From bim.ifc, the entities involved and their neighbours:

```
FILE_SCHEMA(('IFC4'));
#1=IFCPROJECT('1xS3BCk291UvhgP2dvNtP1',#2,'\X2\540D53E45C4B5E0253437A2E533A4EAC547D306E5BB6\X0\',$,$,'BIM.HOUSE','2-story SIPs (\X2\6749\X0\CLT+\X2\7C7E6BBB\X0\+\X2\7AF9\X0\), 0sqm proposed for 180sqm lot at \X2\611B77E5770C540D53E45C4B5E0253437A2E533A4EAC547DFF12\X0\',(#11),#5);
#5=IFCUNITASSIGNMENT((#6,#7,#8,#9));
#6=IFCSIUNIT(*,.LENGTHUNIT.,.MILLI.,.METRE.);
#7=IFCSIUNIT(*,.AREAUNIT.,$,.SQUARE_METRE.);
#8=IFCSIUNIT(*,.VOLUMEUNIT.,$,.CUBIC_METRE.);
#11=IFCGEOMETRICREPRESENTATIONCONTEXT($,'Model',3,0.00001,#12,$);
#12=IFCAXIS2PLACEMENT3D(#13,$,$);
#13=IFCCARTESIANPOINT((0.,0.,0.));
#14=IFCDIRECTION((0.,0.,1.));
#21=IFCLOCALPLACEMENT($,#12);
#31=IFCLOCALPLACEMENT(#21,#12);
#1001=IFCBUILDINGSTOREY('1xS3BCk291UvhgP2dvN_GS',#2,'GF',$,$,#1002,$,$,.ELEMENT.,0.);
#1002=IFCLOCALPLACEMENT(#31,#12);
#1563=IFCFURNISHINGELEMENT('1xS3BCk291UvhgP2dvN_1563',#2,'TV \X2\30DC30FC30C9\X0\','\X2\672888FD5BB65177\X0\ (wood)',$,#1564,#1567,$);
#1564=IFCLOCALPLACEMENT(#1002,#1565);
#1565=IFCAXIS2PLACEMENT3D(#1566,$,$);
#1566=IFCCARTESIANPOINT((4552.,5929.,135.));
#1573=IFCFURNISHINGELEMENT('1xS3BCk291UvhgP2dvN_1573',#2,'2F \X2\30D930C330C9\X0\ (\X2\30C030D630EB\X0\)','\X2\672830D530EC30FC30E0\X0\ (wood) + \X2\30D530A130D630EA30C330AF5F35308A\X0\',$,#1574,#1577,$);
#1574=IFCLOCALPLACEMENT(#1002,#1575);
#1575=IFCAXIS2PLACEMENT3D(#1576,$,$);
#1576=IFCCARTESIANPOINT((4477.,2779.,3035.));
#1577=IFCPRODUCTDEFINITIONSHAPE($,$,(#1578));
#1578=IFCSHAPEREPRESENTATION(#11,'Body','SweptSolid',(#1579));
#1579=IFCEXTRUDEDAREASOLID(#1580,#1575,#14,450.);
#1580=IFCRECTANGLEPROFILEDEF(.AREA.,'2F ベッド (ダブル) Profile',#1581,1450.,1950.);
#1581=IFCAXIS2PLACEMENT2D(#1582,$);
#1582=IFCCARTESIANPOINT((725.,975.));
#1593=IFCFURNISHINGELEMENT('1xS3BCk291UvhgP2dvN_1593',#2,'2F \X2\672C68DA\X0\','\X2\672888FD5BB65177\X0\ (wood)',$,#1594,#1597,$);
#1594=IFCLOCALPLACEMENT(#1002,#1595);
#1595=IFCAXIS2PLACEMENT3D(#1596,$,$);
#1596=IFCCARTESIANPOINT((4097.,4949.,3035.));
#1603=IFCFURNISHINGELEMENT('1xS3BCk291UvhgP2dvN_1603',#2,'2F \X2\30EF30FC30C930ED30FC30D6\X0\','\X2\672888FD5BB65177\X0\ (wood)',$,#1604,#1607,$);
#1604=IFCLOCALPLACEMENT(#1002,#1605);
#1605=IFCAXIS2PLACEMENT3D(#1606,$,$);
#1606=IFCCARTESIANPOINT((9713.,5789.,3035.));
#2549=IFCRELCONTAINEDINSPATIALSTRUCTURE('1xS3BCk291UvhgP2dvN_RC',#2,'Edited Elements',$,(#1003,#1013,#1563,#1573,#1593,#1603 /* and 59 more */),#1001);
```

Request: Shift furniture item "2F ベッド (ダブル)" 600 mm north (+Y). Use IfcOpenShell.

```python
import ifcopenshell
import ifcopenshell.api.geometry
import ifcopenshell.util.placement
import ifcopenshell.util.unit

model = ifcopenshell.open("bim.ifc")
unit_scale = ifcopenshell.util.unit.calculate_unit_scale(model)

item = model.by_guid("1xS3BCk291UvhgP2dvN_1573")
matrix = ifcopenshell.util.placement.get_local_placement(item.ObjectPlacement)
matrix[1, 3] += 0.6 / unit_scale
ifcopenshell.api.geometry.edit_object_placement(model, product=item, matrix=matrix, is_si=False)

print(ifcopenshell.util.placement.get_local_placement(item.ObjectPlacement).round(3) + 0.0)

model.write("bim_rev.ifc")
```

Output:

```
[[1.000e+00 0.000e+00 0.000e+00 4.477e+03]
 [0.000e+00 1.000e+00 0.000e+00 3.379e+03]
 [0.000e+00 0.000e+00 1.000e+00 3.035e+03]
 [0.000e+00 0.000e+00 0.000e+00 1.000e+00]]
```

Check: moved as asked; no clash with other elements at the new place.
